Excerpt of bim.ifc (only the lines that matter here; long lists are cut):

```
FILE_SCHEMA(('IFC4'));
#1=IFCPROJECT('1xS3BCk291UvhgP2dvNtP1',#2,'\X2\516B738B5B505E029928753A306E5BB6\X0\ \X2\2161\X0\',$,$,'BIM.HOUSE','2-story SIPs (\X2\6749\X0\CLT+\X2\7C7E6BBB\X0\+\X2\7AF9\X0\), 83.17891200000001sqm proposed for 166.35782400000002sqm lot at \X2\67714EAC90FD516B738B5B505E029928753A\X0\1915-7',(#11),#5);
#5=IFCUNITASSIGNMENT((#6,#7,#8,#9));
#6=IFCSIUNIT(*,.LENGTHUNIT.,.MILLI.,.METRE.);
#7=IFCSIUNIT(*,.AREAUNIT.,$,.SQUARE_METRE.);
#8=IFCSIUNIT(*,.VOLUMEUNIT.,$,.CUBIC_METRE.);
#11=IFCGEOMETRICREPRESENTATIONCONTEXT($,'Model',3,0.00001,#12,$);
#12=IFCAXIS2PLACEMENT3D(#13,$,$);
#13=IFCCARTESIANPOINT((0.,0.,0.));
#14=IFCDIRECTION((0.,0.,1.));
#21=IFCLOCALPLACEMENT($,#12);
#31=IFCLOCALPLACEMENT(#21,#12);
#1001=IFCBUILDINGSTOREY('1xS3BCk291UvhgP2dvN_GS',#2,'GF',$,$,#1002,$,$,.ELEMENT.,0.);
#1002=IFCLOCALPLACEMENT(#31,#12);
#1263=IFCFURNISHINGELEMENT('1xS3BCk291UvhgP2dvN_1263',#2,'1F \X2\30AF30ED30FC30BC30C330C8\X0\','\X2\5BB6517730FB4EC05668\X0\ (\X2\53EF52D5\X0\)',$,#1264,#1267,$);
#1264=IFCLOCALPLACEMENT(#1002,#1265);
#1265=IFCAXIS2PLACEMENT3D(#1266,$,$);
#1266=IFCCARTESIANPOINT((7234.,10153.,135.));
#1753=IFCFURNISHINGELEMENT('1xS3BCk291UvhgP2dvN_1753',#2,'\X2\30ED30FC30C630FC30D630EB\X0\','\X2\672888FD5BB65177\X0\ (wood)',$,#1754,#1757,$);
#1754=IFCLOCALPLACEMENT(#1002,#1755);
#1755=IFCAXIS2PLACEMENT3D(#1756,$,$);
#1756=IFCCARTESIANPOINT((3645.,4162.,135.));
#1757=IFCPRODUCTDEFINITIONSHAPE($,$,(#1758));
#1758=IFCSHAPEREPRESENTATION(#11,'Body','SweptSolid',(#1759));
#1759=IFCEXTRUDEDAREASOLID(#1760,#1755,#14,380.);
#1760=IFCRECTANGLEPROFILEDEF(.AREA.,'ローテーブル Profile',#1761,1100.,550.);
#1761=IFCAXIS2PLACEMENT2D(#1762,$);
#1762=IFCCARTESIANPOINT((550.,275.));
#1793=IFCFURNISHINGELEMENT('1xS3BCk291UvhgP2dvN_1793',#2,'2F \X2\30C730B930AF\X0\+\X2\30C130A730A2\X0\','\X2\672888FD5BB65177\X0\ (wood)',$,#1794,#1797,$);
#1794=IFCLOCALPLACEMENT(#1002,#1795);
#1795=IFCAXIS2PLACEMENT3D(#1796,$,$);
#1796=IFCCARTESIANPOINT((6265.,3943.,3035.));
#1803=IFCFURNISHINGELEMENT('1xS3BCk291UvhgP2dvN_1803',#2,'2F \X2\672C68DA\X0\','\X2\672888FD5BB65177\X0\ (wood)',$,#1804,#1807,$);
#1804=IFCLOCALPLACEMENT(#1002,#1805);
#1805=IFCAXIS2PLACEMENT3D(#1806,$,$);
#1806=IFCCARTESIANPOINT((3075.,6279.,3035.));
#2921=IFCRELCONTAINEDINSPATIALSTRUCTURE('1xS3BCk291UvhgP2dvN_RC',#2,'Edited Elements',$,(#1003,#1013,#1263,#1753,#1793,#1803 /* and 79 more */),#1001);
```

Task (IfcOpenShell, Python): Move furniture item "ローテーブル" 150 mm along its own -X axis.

```python
import ifcopenshell
import ifcopenshell.api.geometry
import ifcopenshell.util.placement
import ifcopenshell.util.unit

model = ifcopenshell.open("bim.ifc")
unit_scale = ifcopenshell.util.unit.calculate_unit_scale(model)

item = model.by_guid("1xS3BCk291UvhgP2dvN_1753")
matrix = ifcopenshell.util.placement.get_local_placement(item.ObjectPlacement)
matrix[:3, 3] -= matrix[:3, 0] * 0.15 / unit_scale
ifcopenshell.api.geometry.edit_object_placement(model, product=item, matrix=matrix, is_si=False)

print(ifcopenshell.util.placement.get_local_placement(item.ObjectPlacement).round(3) + 0.0)

model.write("bim-out.ifc")
```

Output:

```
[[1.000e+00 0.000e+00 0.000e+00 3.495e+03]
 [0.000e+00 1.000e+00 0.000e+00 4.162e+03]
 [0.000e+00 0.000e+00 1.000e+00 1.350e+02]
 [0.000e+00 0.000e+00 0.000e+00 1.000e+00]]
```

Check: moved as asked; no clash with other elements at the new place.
